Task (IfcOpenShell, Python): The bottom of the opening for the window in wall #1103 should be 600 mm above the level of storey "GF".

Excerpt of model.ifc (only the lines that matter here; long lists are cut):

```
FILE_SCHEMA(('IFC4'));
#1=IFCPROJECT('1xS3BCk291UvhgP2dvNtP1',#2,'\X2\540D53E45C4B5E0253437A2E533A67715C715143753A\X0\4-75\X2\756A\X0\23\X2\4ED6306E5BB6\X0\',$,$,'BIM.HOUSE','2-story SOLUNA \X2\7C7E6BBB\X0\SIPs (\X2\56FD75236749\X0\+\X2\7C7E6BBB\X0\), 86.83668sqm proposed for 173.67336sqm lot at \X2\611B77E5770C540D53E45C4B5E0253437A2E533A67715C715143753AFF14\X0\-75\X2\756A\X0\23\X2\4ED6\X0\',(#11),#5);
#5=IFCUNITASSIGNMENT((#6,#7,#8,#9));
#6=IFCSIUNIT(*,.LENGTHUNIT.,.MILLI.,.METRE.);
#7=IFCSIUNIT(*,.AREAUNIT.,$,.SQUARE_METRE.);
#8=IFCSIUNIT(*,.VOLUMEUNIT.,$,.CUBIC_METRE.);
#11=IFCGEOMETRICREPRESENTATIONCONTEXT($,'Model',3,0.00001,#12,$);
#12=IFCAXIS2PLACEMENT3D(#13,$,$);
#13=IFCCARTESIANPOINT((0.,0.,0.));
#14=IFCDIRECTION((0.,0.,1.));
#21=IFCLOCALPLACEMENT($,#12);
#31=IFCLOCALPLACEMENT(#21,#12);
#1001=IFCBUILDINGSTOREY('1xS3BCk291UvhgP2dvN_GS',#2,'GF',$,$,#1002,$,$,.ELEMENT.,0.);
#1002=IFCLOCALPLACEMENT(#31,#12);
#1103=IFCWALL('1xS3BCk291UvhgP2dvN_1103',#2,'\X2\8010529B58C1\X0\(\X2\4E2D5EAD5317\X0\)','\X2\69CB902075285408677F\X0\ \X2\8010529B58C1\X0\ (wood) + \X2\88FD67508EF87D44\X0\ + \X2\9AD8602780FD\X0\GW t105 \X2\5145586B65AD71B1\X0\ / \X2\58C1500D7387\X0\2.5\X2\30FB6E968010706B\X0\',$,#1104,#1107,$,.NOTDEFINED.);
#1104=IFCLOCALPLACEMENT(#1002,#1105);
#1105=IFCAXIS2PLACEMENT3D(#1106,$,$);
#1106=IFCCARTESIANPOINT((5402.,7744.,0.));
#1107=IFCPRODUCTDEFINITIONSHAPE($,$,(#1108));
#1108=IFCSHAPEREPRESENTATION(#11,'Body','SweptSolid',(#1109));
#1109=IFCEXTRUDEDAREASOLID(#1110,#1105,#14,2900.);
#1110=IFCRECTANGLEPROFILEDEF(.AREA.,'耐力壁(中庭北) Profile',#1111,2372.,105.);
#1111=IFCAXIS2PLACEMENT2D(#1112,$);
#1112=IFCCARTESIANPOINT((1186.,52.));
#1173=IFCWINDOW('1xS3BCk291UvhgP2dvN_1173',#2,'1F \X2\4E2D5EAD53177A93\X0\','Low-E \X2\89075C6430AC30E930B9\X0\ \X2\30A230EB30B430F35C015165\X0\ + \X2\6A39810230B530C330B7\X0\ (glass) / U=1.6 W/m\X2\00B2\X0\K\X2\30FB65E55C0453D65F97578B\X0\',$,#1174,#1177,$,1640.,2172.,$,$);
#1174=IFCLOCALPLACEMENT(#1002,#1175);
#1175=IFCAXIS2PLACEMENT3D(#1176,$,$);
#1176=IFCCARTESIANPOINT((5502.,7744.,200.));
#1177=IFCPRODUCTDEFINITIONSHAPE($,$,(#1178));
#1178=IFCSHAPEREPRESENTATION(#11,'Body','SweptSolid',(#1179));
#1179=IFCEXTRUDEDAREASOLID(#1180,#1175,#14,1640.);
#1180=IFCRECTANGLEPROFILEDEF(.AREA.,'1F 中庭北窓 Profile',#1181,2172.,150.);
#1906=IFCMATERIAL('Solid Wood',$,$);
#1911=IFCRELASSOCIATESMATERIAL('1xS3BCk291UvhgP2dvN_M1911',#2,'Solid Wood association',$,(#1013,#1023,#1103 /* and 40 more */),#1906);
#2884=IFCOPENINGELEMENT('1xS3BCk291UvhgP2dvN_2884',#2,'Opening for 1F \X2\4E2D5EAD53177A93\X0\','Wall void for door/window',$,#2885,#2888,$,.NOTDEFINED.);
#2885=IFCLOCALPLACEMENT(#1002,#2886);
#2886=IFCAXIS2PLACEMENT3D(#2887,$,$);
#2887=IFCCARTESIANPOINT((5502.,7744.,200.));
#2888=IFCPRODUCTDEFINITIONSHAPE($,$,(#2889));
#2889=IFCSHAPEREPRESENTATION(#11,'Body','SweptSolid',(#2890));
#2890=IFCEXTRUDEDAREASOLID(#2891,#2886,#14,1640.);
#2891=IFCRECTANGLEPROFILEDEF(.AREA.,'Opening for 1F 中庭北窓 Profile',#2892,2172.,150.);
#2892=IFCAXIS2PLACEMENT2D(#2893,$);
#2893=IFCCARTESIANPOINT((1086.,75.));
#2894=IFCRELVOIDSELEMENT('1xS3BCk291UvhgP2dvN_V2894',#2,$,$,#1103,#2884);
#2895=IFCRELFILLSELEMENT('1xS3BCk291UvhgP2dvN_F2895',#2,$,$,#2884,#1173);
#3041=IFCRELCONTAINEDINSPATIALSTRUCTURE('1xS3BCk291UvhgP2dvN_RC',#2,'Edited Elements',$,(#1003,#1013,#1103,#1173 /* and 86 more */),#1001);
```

```python
import numpy as np
import ifcopenshell
import ifcopenshell.api.geometry
import ifcopenshell.geom
import ifcopenshell.util.element
import ifcopenshell.util.placement
import ifcopenshell.util.shape
import ifcopenshell.util.unit

model = ifcopenshell.open("model.ifc")
unit_scale = ifcopenshell.util.unit.calculate_unit_scale(model)

window = model.by_guid("1xS3BCk291UvhgP2dvN_1173")
opening = window.FillsVoids[0].RelatingOpeningElement
storey = ifcopenshell.util.element.get_container(window, ifc_class="IfcBuildingStorey")
level = ifcopenshell.util.placement.get_local_placement(storey.ObjectPlacement)[2, 3]

# The opening's origin need not be at the sill, so measure its lowest point.
shape = ifcopenshell.geom.create_shape(ifcopenshell.geom.settings(), opening)
bottom = ifcopenshell.util.shape.get_shape_bottom_elevation(shape, shape.geometry) / unit_scale
dz = level + 600.0 - bottom

shift = np.array([0.0, 0.0, dz])
# The window is not placed relative to its opening, so move both.
for product in (opening, window):
    matrix = ifcopenshell.util.placement.get_local_placement(product.ObjectPlacement)
    matrix[:3, 3] += shift
    ifcopenshell.api.geometry.edit_object_placement(model, product=product, matrix=matrix, is_si=False)

print(f"moved by {dz * unit_scale:+.3f} m")

model.write("model_v2.ifc")
```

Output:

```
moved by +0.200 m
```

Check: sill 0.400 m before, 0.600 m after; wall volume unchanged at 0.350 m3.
